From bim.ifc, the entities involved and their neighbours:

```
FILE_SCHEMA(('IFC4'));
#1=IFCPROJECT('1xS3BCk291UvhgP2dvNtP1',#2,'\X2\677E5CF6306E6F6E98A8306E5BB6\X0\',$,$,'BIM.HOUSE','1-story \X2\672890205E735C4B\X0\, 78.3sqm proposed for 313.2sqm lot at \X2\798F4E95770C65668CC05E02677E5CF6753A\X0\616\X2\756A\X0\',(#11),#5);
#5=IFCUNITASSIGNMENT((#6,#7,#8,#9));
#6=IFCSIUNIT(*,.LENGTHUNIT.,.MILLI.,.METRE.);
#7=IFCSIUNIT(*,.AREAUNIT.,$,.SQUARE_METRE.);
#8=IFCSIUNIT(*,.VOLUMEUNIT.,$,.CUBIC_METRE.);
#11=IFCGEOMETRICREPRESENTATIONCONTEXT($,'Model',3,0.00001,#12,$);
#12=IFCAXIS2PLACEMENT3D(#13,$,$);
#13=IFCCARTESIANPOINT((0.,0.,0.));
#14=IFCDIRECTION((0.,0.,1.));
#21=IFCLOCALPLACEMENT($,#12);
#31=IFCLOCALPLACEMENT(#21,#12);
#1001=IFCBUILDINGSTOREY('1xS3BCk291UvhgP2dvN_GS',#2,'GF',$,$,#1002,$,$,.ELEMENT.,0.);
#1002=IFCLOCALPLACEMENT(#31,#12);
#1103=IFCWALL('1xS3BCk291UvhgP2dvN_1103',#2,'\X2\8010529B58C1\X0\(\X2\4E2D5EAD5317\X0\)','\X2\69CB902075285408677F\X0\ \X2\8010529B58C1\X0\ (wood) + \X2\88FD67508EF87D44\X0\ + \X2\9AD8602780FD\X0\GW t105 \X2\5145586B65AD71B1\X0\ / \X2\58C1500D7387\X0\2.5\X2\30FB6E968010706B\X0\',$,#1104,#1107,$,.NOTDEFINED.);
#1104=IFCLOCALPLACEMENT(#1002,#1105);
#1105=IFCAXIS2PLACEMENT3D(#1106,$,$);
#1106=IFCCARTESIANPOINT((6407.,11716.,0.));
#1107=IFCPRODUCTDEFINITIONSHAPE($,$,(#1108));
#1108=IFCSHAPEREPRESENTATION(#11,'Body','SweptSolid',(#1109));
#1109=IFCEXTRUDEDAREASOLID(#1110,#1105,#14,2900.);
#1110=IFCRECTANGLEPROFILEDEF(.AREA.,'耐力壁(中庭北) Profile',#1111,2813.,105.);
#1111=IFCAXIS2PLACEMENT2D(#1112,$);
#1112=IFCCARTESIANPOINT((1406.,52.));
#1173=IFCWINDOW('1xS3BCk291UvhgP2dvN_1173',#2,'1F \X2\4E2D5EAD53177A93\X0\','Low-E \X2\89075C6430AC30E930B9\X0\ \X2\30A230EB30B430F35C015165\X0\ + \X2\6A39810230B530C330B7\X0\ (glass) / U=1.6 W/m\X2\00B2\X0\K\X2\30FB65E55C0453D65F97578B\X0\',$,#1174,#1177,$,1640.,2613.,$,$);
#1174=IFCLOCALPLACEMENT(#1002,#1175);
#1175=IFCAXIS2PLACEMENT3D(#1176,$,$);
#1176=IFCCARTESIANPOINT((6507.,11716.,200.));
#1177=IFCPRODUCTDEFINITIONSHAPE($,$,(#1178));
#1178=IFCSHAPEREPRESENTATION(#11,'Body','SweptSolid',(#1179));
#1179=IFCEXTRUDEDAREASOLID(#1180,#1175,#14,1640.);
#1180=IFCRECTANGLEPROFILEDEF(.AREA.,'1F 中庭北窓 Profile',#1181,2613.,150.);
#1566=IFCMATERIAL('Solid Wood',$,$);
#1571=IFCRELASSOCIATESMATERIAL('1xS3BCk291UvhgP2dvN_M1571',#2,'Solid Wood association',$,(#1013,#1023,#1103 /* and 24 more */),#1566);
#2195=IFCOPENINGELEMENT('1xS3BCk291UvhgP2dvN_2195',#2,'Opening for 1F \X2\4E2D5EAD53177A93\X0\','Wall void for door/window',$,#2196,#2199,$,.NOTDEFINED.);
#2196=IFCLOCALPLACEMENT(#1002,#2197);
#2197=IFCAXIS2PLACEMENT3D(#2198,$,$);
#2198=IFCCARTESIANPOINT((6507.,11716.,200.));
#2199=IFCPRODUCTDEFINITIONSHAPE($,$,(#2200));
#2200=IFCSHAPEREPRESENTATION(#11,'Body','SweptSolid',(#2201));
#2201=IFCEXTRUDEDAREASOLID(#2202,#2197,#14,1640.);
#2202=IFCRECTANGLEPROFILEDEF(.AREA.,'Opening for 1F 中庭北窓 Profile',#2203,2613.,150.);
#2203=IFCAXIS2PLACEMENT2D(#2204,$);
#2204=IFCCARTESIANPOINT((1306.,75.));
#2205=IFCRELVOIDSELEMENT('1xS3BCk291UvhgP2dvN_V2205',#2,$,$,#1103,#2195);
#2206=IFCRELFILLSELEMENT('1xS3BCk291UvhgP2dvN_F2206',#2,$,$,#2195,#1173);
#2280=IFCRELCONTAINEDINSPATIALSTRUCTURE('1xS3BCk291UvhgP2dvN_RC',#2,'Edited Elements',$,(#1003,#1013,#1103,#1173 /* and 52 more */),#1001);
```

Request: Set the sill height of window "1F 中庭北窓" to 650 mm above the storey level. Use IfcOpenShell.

```python
import numpy as np
import ifcopenshell
import ifcopenshell.api.geometry
import ifcopenshell.geom
import ifcopenshell.util.element
import ifcopenshell.util.placement
import ifcopenshell.util.shape
import ifcopenshell.util.unit

model = ifcopenshell.open("bim.ifc")
unit_scale = ifcopenshell.util.unit.calculate_unit_scale(model)

window = model.by_guid("1xS3BCk291UvhgP2dvN_1173")
opening = window.FillsVoids[0].RelatingOpeningElement
storey = ifcopenshell.util.element.get_container(window, ifc_class="IfcBuildingStorey")
level = ifcopenshell.util.placement.get_local_placement(storey.ObjectPlacement)[2, 3]

# The opening's origin need not be at the sill, so measure its lowest point.
shape = ifcopenshell.geom.create_shape(ifcopenshell.geom.settings(), opening)
bottom = ifcopenshell.util.shape.get_shape_bottom_elevation(shape, shape.geometry) / unit_scale
dz = level + 650.0 - bottom

shift = np.array([0.0, 0.0, dz])
# The window is not placed relative to its opening, so move both.
for product in (opening, window):
    matrix = ifcopenshell.util.placement.get_local_placement(product.ObjectPlacement)
    matrix[:3, 3] += shift
    ifcopenshell.api.geometry.edit_object_placement(model, product=product, matrix=matrix, is_si=False)

print(f"moved by {dz * unit_scale:+.3f} m")

model.write("bim-out.ifc")
```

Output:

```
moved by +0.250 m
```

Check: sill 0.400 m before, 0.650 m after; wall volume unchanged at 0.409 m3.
